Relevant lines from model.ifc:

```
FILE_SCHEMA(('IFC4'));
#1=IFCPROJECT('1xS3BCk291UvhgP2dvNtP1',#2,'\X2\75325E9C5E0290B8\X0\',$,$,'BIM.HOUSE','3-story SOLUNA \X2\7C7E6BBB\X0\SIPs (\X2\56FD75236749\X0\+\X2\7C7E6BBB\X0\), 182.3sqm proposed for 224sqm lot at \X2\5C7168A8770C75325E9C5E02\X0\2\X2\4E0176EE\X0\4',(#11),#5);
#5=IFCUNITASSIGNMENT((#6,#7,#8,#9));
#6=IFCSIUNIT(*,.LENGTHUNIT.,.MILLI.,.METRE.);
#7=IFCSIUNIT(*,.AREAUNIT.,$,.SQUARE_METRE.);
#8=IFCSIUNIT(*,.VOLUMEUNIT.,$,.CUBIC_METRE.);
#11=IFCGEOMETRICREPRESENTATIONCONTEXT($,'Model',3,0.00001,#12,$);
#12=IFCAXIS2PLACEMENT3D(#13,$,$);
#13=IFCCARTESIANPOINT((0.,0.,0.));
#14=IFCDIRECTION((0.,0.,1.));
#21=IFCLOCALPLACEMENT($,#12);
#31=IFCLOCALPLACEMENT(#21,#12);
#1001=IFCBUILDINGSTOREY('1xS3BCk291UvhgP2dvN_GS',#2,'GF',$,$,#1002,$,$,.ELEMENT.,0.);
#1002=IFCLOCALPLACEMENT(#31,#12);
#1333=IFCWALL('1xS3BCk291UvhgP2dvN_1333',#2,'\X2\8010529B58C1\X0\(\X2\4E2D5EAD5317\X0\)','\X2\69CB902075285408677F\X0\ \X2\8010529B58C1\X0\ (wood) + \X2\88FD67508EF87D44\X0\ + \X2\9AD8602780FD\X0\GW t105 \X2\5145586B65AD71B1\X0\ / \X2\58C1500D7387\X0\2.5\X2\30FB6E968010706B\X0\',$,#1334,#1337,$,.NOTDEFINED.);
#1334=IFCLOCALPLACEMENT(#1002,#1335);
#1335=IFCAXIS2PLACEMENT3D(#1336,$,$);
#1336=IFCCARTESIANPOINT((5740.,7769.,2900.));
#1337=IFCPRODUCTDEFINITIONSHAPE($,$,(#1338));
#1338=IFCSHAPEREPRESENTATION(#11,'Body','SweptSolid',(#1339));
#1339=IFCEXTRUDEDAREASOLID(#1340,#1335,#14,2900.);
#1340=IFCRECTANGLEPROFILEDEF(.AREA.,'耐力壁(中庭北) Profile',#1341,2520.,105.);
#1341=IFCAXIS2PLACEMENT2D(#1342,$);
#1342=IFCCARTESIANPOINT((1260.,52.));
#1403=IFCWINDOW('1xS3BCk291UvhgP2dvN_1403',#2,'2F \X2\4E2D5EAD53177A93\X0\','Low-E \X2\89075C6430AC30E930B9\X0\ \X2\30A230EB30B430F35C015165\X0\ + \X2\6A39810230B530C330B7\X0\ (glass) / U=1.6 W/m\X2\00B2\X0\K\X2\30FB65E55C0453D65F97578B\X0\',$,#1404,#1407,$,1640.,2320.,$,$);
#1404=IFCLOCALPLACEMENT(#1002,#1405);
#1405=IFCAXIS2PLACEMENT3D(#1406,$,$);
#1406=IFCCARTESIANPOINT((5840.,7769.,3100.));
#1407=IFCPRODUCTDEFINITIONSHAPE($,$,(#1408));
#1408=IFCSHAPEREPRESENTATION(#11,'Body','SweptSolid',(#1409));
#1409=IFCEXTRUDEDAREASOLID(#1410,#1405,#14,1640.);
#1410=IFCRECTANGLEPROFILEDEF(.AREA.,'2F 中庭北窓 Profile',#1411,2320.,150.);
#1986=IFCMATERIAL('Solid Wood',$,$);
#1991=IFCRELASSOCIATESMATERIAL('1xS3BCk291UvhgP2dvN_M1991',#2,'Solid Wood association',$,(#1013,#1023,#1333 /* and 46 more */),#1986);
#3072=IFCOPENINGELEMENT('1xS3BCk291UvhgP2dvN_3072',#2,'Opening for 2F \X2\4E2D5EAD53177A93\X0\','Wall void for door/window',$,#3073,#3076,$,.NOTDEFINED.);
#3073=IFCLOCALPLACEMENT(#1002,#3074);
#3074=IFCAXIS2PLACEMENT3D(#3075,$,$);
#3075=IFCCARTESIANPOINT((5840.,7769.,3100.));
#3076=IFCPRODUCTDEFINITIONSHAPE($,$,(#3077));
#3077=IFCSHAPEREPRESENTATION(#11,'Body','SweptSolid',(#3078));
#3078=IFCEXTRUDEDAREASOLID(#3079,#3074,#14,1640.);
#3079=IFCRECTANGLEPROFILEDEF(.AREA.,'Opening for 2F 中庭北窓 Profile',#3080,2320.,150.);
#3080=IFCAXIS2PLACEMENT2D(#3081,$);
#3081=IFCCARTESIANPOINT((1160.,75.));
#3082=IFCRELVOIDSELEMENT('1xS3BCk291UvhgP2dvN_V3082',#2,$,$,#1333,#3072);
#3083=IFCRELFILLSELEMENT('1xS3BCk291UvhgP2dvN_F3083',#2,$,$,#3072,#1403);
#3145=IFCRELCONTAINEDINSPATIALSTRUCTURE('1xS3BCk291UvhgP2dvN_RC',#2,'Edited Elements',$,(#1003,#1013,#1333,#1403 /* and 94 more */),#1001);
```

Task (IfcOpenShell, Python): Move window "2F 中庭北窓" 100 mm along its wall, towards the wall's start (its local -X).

```python
import ifcopenshell
import ifcopenshell.api.geometry
import ifcopenshell.util.placement

model = ifcopenshell.open("model.ifc")

window = model.by_id(1403)
opening = window.FillsVoids[0].RelatingOpeningElement
wall = opening.VoidsElements[0].RelatingBuildingElement

wall_matrix = ifcopenshell.util.placement.get_local_placement(wall.ObjectPlacement)
shift = wall_matrix[:3, 0] * -100.0
before = ifcopenshell.util.placement.get_local_placement(window.ObjectPlacement)[:3, 3].copy()

# The window is not placed relative to its opening, so move both.
for product in (opening, window):
    matrix = ifcopenshell.util.placement.get_local_placement(product.ObjectPlacement)
    matrix[:3, 3] += shift
    ifcopenshell.api.geometry.edit_object_placement(model, product=product, matrix=matrix, is_si=False)

after = ifcopenshell.util.placement.get_local_placement(window.ObjectPlacement)[:3, 3]
print("window moved by", (after - before).round(3) + 0.0)

model.write("model_v2.ifc")
```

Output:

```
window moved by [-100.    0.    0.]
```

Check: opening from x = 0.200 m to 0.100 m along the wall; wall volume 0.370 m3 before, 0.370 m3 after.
